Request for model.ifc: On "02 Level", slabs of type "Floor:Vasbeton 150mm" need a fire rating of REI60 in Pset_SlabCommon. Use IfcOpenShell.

First a look at what the model holds.

```python
import ifcopenshell
import ifcopenshell.util.element

model = ifcopenshell.open("model.ifc")
print(model.schema)
storey = next(s for s in model.by_type("IfcBuildingStorey") if s.Name == "02 Level")
slabs = [e for e in ifcopenshell.util.element.get_decomposition(storey) if e.is_a("IfcSlab")]
seen = {}
for e in slabs:
    element_type = ifcopenshell.util.element.get_type(e)
    key = (element_type.Name if element_type != e and element_type else None, ifcopenshell.util.element.get_pset(e, "Pset_SlabCommon", "FireRating"))
    seen[key] = seen.get(key, 0) + 1
for (name, value), count in sorted(seen.items(), key=str):
    print(count, "x", name, "|", value)
```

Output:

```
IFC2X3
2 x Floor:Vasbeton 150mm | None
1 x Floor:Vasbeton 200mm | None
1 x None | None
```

```python
import ifcopenshell
import ifcopenshell.api.pset
import ifcopenshell.util.element

model = ifcopenshell.open("model.ifc")

storey = next(s for s in model.by_type("IfcBuildingStorey") if s.Name == "02 Level")
slabs = [e for e in ifcopenshell.util.element.get_decomposition(storey) if e.is_a("IfcSlab")]

count = 0
for e in slabs:
    element_type = ifcopenshell.util.element.get_type(e)
    if element_type in (None, e) or element_type.Name != "Floor:Vasbeton 150mm":
        continue
    # add_pset returns the element's existing set when there is one.
    pset = ifcopenshell.api.pset.add_pset(model, product=e, name="Pset_SlabCommon")
    ifcopenshell.api.pset.edit_pset(model, pset=pset, properties={"FireRating": "REI60"})
    count += 1

print(count, "slabs updated")

model.write("model_rev.ifc")
```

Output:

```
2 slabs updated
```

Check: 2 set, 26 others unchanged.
